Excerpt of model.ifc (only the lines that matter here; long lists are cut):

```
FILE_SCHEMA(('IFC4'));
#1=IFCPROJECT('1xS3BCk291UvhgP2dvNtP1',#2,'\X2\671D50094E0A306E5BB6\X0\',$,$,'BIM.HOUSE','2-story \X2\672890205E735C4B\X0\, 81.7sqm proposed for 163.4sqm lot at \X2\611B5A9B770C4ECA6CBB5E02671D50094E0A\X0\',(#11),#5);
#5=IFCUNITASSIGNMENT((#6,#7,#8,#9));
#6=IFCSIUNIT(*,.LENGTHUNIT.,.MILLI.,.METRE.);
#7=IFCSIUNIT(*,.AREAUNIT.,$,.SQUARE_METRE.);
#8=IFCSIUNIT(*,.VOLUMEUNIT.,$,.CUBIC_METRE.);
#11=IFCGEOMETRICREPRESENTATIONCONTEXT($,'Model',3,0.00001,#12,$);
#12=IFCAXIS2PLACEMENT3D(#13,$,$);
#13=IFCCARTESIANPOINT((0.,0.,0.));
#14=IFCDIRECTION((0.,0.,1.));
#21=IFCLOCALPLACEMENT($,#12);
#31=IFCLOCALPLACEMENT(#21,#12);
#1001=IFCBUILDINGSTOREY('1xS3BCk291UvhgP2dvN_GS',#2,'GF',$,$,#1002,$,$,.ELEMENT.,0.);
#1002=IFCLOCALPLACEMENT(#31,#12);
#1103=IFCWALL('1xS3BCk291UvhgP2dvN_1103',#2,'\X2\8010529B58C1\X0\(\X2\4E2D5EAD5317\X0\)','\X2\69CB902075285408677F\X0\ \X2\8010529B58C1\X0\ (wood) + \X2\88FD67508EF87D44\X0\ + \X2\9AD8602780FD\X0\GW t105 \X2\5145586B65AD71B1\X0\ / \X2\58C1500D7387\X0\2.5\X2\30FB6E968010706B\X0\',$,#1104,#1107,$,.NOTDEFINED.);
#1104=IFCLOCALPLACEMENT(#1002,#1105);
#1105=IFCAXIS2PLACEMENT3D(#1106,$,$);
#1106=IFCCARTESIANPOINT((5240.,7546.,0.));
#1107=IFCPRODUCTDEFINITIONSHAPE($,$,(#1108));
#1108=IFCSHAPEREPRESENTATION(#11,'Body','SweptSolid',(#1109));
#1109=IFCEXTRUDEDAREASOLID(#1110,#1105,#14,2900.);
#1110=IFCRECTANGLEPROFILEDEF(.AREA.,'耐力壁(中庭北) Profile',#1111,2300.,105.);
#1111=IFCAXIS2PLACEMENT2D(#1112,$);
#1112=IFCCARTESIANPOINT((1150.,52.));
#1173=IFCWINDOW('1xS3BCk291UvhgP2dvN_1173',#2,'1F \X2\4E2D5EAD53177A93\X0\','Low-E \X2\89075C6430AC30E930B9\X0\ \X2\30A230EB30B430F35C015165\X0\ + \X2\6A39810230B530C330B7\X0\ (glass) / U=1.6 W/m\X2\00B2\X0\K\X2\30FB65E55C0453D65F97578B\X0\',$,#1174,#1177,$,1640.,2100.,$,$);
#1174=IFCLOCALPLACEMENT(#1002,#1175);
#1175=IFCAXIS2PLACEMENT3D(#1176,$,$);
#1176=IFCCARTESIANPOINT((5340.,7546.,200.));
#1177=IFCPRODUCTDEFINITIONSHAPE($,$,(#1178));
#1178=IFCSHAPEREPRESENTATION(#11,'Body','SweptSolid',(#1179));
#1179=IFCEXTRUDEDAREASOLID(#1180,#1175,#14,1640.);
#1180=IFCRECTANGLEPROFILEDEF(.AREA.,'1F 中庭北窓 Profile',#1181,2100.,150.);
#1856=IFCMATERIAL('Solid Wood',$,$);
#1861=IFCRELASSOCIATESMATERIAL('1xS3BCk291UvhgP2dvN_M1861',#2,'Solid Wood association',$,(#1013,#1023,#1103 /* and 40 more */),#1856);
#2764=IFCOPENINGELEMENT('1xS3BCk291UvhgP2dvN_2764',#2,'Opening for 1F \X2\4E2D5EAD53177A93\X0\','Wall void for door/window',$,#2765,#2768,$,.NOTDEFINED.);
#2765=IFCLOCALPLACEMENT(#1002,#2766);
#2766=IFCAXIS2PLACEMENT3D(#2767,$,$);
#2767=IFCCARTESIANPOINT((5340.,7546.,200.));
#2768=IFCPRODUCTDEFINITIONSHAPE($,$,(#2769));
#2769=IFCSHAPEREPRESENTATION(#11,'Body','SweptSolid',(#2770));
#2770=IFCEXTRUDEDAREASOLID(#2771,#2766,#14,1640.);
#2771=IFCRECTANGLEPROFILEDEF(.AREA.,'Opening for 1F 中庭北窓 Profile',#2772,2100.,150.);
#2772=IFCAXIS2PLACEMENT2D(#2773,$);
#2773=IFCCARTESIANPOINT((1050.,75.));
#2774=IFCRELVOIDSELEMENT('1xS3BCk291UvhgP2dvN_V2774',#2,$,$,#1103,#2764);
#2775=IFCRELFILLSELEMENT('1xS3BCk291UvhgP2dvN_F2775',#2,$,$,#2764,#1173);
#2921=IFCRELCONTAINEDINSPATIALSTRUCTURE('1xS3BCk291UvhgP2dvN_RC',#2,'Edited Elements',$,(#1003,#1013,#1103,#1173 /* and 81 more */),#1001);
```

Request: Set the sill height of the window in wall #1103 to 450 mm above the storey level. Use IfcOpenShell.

```python
import numpy as np
import ifcopenshell
import ifcopenshell.api.geometry
import ifcopenshell.geom
import ifcopenshell.util.element
import ifcopenshell.util.placement
import ifcopenshell.util.shape
import ifcopenshell.util.unit

model = ifcopenshell.open("model.ifc")
unit_scale = ifcopenshell.util.unit.calculate_unit_scale(model)

window = model.by_id(1173)
opening = window.FillsVoids[0].RelatingOpeningElement
storey = ifcopenshell.util.element.get_container(window, ifc_class="IfcBuildingStorey")
level = ifcopenshell.util.placement.get_local_placement(storey.ObjectPlacement)[2, 3]

# The opening's origin need not be at the sill, so measure its lowest point.
shape = ifcopenshell.geom.create_shape(ifcopenshell.geom.settings(), opening)
bottom = ifcopenshell.util.shape.get_shape_bottom_elevation(shape, shape.geometry) / unit_scale
dz = level + 450.0 - bottom

shift = np.array([0.0, 0.0, dz])
# The window is not placed relative to its opening, so move both.
for product in (opening, window):
    matrix = ifcopenshell.util.placement.get_local_placement(product.ObjectPlacement)
    matrix[:3, 3] += shift
    ifcopenshell.api.geometry.edit_object_placement(model, product=product, matrix=matrix, is_si=False)

print(f"moved by {dz * unit_scale:+.3f} m")

model.write("model-out.ifc")
```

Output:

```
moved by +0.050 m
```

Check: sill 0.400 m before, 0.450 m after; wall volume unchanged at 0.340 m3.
